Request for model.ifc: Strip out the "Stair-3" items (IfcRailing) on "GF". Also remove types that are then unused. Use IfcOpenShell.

First a look at what the model holds.

```python
import ifcopenshell
import ifcopenshell.util.element

model = ifcopenshell.open("model.ifc")
print(model.schema)
storey = next(s for s in model.by_type("IfcBuildingStorey") if s.Name == "GF")
railings = [e for e in ifcopenshell.util.element.get_decomposition(storey) if e.is_a("IfcRailing")]
seen = {}
for e in railings:
    element_type = ifcopenshell.util.element.get_type(e)
    name = element_type.Name if element_type not in (None, e) else None
    seen[name] = seen.get(name, 0) + 1
for name, count in sorted(seen.items(), key=str):
    print(count, "x", name)
```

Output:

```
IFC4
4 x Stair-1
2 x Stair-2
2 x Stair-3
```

```python
import ifcopenshell
import ifcopenshell.api.root
import ifcopenshell.util.element

model = ifcopenshell.open("model.ifc")

storey = next(s for s in model.by_type("IfcBuildingStorey") if s.Name == "GF")
railings = [e for e in ifcopenshell.util.element.get_decomposition(storey) if e.is_a("IfcRailing")]
targets = [e for e in railings if (t := ifcopenshell.util.element.get_type(e)) not in (None, e) and t.Name == "Stair-3"]
types = {ifcopenshell.util.element.get_type(e) for e in targets} - {None, *targets}

for e in targets:
    ifcopenshell.api.root.remove_product(model, product=e)
print(len(targets), "removed")

unused = [t for t in types if not ifcopenshell.util.element.get_types(t)]
for t in unused:
    ifcopenshell.api.root.remove_product(model, product=t)
print(len(unused), "unused types removed")

model.write("model_rev.ifc")
```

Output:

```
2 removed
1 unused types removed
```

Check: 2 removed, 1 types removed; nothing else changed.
